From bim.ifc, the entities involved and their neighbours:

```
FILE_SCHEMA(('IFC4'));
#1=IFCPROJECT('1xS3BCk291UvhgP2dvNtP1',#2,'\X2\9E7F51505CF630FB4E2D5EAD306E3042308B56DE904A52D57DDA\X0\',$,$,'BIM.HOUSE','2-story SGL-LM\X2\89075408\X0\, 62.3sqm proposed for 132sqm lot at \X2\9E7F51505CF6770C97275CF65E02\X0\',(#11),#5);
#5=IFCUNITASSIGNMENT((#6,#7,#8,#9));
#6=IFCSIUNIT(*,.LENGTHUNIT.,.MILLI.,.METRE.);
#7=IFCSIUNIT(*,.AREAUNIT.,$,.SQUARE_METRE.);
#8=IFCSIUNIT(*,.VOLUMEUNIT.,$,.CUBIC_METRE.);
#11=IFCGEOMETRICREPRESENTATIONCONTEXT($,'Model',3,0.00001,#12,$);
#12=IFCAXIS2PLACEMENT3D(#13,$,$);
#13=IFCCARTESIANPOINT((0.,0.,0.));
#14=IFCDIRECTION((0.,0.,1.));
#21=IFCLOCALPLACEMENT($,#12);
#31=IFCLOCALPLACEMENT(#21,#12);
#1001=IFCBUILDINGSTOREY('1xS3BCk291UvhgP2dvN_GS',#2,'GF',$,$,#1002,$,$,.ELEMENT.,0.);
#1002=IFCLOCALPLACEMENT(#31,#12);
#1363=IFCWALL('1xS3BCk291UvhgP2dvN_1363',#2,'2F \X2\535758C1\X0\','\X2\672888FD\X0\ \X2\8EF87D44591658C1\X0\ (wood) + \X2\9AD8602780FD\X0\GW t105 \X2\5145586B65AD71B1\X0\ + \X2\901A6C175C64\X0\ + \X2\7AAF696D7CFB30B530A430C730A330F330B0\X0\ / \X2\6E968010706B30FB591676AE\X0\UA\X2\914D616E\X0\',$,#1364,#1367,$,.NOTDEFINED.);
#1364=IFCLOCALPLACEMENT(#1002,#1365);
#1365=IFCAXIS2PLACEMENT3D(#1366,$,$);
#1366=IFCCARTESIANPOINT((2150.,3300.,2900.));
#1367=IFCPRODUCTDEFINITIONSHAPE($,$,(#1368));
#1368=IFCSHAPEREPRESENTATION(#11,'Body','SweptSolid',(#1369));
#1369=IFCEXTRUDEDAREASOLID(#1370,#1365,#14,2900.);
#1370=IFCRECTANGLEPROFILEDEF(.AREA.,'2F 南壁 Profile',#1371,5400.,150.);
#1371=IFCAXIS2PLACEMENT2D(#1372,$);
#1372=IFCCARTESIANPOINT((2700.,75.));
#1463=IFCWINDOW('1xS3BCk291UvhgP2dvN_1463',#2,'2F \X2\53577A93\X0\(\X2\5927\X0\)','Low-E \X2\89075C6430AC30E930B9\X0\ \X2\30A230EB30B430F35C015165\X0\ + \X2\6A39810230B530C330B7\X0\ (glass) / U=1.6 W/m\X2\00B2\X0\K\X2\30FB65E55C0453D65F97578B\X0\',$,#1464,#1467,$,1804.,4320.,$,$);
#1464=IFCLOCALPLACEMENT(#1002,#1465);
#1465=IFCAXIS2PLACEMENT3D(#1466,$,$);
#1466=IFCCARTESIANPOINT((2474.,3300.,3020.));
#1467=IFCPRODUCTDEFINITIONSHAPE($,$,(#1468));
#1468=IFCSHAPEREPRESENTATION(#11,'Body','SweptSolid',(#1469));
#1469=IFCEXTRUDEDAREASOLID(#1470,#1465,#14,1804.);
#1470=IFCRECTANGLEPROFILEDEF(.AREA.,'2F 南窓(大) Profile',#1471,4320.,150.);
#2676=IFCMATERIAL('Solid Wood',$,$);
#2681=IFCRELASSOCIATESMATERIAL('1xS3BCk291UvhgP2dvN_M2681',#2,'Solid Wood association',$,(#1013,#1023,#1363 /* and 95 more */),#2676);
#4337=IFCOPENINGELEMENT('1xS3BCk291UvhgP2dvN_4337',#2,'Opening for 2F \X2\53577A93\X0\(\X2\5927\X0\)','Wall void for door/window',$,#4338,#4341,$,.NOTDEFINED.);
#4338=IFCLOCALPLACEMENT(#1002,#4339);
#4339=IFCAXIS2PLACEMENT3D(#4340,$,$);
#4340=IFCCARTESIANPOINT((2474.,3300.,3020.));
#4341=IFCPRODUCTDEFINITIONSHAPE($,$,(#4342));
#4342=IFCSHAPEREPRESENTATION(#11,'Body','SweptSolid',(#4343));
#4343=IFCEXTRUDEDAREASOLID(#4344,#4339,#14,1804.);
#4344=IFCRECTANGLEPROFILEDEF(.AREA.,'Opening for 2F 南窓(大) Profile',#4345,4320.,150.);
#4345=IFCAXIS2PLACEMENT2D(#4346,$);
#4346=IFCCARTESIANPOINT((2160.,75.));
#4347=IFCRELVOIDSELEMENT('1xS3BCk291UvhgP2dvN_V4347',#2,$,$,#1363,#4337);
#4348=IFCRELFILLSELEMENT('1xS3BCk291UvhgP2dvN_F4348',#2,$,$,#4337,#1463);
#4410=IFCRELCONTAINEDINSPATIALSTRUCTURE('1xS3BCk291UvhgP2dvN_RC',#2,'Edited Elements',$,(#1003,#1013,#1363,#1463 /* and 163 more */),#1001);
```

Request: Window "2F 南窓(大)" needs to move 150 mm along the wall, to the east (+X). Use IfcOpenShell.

```python
import ifcopenshell
import ifcopenshell.api.geometry
import ifcopenshell.util.placement
import ifcopenshell.util.unit

model = ifcopenshell.open("bim.ifc")
unit_scale = ifcopenshell.util.unit.calculate_unit_scale(model)

window = model.by_id(1463)
opening = window.FillsVoids[0].RelatingOpeningElement
wall = opening.VoidsElements[0].RelatingBuildingElement

wall_matrix = ifcopenshell.util.placement.get_local_placement(wall.ObjectPlacement)
shift = wall_matrix[:3, 0] * 0.15 / unit_scale
before = ifcopenshell.util.placement.get_local_placement(window.ObjectPlacement)[:3, 3].copy()

# The window is not placed relative to its opening, so move both.
for product in (opening, window):
    matrix = ifcopenshell.util.placement.get_local_placement(product.ObjectPlacement)
    matrix[:3, 3] += shift
    ifcopenshell.api.geometry.edit_object_placement(model, product=product, matrix=matrix, is_si=False)

after = ifcopenshell.util.placement.get_local_placement(window.ObjectPlacement)[:3, 3]
print("window moved by", (after - before).round(3) + 0.0)

model.write("bim_v2.ifc")
```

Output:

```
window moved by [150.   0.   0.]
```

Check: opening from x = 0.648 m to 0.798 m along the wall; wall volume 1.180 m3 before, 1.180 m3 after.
